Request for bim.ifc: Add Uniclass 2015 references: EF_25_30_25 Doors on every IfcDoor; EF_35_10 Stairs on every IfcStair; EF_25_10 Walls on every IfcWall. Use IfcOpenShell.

First a look at what the model holds.

```python
import ifcopenshell

model = ifcopenshell.open("bim.ifc")
print(model.schema)
print("classifications:", [c.Name for c in model.by_type("IfcClassification")])
for ifc_class in ("IfcDoor", "IfcRoof", "IfcStair", "IfcWall", "IfcWindow"):
    print(ifc_class, len(model.by_type(ifc_class)))
```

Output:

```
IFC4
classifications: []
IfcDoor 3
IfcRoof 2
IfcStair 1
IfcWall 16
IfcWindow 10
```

```python
import ifcopenshell
import ifcopenshell.api.classification

model = ifcopenshell.open("bim.ifc")

system = ifcopenshell.api.classification.add_classification(model, classification="Uniclass 2015")

codes = {
    "IfcDoor": ("EF_25_30_25", "Doors"),
    "IfcStair": ("EF_35_10", "Stairs"),
    "IfcWall": ("EF_25_10", "Walls"),
}
for ifc_class, (code, name) in codes.items():
    products = model.by_type(ifc_class)
    ifcopenshell.api.classification.add_reference(
        model, products=products, classification=system, identification=code, name=name
    )
    print(code, len(products))

model.write("bim_edited.ifc")
```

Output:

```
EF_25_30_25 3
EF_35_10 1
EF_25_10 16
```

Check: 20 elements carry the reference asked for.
